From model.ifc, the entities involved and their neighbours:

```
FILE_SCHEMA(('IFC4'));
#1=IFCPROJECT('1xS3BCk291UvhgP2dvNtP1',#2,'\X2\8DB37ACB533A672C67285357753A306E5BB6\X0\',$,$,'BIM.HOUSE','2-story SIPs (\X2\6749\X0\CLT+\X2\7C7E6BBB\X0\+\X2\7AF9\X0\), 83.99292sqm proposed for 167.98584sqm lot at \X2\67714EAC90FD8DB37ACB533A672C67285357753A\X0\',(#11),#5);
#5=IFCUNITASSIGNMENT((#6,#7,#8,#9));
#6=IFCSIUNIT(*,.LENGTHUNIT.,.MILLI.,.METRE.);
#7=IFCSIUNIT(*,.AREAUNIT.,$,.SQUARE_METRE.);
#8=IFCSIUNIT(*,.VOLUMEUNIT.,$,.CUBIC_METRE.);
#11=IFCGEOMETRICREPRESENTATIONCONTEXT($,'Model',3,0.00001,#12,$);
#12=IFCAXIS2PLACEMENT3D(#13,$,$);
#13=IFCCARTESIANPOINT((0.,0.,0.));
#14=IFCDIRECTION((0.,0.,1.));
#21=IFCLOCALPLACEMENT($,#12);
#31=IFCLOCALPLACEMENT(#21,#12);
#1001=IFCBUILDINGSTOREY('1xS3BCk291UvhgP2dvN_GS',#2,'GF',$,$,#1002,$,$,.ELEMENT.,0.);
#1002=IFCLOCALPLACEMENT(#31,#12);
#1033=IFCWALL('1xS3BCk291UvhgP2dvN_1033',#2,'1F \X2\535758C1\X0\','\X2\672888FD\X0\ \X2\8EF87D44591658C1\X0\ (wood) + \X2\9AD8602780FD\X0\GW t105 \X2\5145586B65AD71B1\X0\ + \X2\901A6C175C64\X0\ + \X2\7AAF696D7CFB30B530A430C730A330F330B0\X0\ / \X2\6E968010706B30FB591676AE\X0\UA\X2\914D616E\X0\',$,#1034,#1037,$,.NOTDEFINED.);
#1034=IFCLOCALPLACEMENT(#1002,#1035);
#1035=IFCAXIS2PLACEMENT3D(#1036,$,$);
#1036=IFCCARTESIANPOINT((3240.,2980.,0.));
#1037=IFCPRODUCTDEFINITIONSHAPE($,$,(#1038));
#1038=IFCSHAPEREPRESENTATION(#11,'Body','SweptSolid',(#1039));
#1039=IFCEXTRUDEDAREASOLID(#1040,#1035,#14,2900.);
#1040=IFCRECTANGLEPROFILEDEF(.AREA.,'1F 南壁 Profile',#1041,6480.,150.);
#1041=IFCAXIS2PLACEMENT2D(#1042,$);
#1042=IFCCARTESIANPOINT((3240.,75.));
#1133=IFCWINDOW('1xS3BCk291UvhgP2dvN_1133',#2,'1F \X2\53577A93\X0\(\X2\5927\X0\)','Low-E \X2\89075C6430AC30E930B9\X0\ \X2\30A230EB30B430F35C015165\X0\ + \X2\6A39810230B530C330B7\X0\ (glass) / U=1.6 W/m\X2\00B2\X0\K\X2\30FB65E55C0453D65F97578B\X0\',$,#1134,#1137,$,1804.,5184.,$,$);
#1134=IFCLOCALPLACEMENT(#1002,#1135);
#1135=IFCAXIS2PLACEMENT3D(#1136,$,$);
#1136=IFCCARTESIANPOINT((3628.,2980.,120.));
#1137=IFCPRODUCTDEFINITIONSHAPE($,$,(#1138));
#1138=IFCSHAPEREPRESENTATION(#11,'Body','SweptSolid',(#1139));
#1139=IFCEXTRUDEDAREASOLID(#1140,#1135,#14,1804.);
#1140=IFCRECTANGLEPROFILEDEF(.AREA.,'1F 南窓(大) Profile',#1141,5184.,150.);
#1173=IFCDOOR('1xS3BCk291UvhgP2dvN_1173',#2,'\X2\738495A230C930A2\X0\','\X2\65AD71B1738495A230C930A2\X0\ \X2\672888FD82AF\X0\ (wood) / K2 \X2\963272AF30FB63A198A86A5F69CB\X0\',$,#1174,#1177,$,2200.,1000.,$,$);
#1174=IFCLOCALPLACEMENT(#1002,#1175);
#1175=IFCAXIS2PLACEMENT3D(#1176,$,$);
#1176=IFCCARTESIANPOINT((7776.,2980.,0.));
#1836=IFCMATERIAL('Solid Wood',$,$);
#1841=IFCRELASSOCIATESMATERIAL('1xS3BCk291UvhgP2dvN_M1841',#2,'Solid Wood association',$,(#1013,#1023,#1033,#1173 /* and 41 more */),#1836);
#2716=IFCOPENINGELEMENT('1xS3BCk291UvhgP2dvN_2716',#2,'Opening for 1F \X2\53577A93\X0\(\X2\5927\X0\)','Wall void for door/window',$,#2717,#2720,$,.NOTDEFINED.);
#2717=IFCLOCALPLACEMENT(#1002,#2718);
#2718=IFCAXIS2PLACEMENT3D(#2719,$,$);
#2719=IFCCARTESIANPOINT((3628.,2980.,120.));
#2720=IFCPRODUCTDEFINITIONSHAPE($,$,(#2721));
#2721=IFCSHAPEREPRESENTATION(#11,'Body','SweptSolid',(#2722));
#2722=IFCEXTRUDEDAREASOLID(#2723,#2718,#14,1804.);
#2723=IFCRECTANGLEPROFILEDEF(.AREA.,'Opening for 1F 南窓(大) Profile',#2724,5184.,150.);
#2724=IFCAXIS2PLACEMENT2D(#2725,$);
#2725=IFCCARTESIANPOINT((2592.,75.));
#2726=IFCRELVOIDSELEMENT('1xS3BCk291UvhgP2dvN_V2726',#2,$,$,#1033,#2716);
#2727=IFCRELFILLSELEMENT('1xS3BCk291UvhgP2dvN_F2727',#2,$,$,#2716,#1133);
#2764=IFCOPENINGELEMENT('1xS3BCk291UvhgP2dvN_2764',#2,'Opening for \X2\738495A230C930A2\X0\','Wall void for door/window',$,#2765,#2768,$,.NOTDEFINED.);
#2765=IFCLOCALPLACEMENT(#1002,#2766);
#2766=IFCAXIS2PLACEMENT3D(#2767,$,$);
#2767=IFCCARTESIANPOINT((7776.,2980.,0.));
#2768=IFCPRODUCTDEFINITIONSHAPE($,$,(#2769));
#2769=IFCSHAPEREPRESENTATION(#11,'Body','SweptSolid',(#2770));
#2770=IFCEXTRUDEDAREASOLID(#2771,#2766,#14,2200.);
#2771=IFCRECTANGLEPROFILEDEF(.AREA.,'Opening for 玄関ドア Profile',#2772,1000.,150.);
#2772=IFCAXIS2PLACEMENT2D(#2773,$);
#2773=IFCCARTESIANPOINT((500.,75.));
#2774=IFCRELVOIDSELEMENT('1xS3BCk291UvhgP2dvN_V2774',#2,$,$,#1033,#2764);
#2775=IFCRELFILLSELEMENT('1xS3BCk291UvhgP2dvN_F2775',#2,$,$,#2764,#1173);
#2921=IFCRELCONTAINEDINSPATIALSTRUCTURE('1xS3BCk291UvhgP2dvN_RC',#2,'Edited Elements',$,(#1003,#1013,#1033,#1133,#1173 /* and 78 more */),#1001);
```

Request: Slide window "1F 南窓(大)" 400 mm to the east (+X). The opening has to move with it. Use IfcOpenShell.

```python
import ifcopenshell
import ifcopenshell.api.geometry
import ifcopenshell.util.placement

model = ifcopenshell.open("model.ifc")

window = model.by_guid("1xS3BCk291UvhgP2dvN_1133")
opening = window.FillsVoids[0].RelatingOpeningElement
wall = opening.VoidsElements[0].RelatingBuildingElement

wall_matrix = ifcopenshell.util.placement.get_local_placement(wall.ObjectPlacement)
shift = wall_matrix[:3, 0] * 400.0
before = ifcopenshell.util.placement.get_local_placement(window.ObjectPlacement)[:3, 3].copy()

# The window is not placed relative to its opening, so move both.
for product in (opening, window):
    matrix = ifcopenshell.util.placement.get_local_placement(product.ObjectPlacement)
    matrix[:3, 3] += shift
    ifcopenshell.api.geometry.edit_object_placement(model, product=product, matrix=matrix, is_si=False)

after = ifcopenshell.util.placement.get_local_placement(window.ObjectPlacement)[:3, 3]
print("window moved by", (after - before).round(3) + 0.0)

model.write("model_v2.ifc")
```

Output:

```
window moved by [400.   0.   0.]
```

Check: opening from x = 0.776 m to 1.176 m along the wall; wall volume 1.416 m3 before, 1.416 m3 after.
